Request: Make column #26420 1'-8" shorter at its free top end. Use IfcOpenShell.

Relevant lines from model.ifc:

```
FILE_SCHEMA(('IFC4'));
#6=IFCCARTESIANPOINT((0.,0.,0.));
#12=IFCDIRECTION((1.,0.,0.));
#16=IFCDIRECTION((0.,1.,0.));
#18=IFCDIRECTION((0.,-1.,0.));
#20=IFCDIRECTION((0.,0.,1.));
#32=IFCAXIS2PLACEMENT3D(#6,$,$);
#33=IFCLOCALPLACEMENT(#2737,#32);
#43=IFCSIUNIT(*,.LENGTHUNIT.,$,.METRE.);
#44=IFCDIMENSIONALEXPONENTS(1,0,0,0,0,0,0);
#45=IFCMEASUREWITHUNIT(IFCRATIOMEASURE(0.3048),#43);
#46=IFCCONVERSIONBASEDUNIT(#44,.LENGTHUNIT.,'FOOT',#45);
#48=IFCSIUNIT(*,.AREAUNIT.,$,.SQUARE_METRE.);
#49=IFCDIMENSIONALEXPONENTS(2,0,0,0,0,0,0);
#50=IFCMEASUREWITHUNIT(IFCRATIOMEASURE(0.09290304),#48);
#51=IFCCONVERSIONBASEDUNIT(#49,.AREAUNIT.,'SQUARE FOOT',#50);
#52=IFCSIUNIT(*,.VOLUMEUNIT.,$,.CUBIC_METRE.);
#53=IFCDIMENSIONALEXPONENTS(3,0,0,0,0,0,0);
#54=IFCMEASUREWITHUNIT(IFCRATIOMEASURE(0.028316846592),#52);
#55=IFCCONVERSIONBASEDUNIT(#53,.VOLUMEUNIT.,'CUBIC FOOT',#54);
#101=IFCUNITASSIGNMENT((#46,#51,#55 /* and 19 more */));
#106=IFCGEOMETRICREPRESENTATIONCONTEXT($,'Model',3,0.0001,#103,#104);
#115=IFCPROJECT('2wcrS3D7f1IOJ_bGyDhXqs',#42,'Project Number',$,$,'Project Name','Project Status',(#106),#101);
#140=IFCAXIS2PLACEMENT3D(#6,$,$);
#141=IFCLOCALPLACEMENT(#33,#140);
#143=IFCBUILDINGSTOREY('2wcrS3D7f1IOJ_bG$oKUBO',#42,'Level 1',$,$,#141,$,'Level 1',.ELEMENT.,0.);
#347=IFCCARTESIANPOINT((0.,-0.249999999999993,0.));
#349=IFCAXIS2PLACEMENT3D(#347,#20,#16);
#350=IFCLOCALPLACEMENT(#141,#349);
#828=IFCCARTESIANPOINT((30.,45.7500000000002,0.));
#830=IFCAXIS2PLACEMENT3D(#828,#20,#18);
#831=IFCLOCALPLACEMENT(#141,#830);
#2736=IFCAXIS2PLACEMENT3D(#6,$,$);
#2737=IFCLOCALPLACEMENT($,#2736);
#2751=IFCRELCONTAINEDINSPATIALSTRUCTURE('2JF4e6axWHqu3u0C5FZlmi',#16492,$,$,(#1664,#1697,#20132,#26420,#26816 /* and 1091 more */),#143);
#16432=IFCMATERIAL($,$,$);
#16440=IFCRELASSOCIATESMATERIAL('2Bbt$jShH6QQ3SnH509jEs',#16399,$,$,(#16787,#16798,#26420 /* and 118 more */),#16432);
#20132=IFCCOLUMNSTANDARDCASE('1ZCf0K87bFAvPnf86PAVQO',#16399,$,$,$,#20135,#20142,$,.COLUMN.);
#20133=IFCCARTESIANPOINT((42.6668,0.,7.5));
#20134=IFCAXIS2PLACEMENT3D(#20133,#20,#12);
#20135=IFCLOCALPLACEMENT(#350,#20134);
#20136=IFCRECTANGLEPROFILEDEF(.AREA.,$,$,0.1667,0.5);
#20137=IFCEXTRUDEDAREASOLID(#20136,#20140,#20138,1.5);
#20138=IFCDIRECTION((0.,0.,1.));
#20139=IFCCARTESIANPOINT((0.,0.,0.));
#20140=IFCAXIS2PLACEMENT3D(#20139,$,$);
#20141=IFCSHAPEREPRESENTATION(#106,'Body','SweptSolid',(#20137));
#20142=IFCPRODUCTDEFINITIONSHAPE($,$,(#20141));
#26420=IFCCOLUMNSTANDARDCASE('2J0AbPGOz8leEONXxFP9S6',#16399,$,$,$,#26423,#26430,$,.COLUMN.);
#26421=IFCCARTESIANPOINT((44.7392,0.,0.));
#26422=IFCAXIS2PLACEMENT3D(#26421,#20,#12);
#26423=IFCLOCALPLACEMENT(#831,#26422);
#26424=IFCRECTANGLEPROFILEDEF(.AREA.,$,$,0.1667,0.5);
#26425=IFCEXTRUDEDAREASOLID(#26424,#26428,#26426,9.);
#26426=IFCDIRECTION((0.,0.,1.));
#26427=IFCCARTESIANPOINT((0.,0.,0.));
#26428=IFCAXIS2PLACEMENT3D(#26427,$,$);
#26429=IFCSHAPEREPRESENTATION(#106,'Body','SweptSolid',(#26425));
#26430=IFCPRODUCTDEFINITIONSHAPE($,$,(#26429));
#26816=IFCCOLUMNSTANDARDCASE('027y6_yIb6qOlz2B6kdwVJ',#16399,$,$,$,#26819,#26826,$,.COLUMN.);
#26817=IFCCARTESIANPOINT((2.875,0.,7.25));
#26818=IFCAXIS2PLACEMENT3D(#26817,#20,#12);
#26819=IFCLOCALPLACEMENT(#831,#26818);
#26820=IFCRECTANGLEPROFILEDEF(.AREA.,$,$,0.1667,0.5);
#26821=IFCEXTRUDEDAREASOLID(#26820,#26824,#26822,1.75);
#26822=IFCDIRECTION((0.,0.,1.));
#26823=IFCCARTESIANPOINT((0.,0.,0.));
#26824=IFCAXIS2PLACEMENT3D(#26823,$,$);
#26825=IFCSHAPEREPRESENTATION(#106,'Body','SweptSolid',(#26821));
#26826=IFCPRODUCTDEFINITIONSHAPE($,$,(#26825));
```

```python
import ifcopenshell
import ifcopenshell.util.unit

model = ifcopenshell.open("model.ifc")
unit_scale = ifcopenshell.util.unit.calculate_unit_scale(model)

member = model.by_guid("2J0AbPGOz8leEONXxFP9S6")
change = -20 * 0.0254 / unit_scale

# The extrusion runs towards the end named, so only its depth changes.
body = next(r for r in member.Representation.Representations if r.RepresentationIdentifier == "Body")
solid = body.Items[0]
old_length = solid.Depth
solid.Depth += change

print(f"length {old_length:g} -> {solid.Depth:g}")

model.write("model_edited.ifc")
```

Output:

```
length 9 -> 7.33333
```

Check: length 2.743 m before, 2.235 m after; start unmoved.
